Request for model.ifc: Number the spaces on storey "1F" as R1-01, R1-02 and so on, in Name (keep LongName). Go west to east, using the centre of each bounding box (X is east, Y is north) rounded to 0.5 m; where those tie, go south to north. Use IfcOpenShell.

First a look at what the model holds.

```python
import ifcopenshell
import ifcopenshell.util.element
import ifcopenshell.util.placement

model = ifcopenshell.open("model.ifc")
print(model.schema)
storey = next(s for s in model.by_type("IfcBuildingStorey") if s.Name == "1F")
spaces = [e for e in ifcopenshell.util.element.get_decomposition(storey) if e.is_a("IfcSpace")]
for e in sorted(spaces, key=lambda e: e.id()):
    origin = ifcopenshell.util.placement.get_local_placement(e.ObjectPlacement)[:3, 3]
    print(e.id(), e.Name, e.LongName, origin.round(2) + 0.0, sep=" | ")
```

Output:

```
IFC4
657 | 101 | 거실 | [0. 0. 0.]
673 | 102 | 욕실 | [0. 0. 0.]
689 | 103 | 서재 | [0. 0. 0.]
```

```python
import ifcopenshell
import ifcopenshell.geom
import ifcopenshell.util.element
import ifcopenshell.util.shape

model = ifcopenshell.open("model.ifc")
settings = ifcopenshell.geom.settings()
settings.set("use-world-coords", True)


def centre(element):
    shape = ifcopenshell.geom.create_shape(settings, element)
    return ifcopenshell.util.shape.get_bbox_centroid(shape.geometry)


storey = next(s for s in model.by_type("IfcBuildingStorey") if s.Name == "1F")
spaces = [e for e in ifcopenshell.util.element.get_decomposition(storey) if e.is_a("IfcSpace")]

# Insertion points can sit at a corner or the storey origin, so sort by the geometry (in metres).
centres = {e: centre(e) for e in spaces}
spaces.sort(key=lambda e: (round(centres[e][0] / 0.5), centres[e][1]))

for i, e in enumerate(spaces, start=1):
    number = f"R1-{i:02d}"
    e.Name = number
    print(e.id(), number)

model.write("model_rev.ifc")
```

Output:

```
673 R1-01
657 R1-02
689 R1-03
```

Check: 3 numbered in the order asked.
